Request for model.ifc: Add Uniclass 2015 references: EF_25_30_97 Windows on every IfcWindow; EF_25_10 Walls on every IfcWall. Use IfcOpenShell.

First a look at what the model holds.

```python
import ifcopenshell

model = ifcopenshell.open("model.ifc")
print(model.schema)
print("classifications:", [c.Name for c in model.by_type("IfcClassification")])
for ifc_class in ("IfcDoor", "IfcRoof", "IfcStair", "IfcWall", "IfcWindow"):
    print(ifc_class, len(model.by_type(ifc_class)))
```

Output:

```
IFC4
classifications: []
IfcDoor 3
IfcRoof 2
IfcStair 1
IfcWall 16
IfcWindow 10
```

```python
import ifcopenshell
import ifcopenshell.api.classification

model = ifcopenshell.open("model.ifc")

system = ifcopenshell.api.classification.add_classification(model, classification="Uniclass 2015")

codes = {
    "IfcWindow": ("EF_25_30_97", "Windows"),
    "IfcWall": ("EF_25_10", "Walls"),
}
for ifc_class, (code, name) in codes.items():
    products = model.by_type(ifc_class)
    ifcopenshell.api.classification.add_reference(
        model, products=products, classification=system, identification=code, name=name
    )
    print(code, len(products))

model.write("model_updated.ifc")
```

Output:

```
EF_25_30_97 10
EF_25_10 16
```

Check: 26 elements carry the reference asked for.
